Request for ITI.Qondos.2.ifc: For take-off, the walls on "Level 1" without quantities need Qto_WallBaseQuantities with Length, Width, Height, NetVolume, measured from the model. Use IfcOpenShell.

First a look at what the model holds.

```python
import ifcopenshell
import ifcopenshell.util.element
import ifcopenshell.util.unit

model = ifcopenshell.open("ITI.Qondos.2.ifc")
print(model.schema)
for unit_type in ("LENGTHUNIT", "AREAUNIT", "VOLUMEUNIT"):
    print(unit_type, ifcopenshell.util.unit.calculate_unit_scale(model, unit_type))
storey = next(s for s in model.by_type("IfcBuildingStorey") if s.Name == "Level 1")
walls = [e for e in ifcopenshell.util.element.get_decomposition(storey) if e.is_a("IfcWall")]
for e in sorted(walls, key=lambda e: e.id()):
    print(e.id(), e.is_a(), e.Name, list(ifcopenshell.util.element.get_psets(e, qtos_only=True)), sep=" | ")
```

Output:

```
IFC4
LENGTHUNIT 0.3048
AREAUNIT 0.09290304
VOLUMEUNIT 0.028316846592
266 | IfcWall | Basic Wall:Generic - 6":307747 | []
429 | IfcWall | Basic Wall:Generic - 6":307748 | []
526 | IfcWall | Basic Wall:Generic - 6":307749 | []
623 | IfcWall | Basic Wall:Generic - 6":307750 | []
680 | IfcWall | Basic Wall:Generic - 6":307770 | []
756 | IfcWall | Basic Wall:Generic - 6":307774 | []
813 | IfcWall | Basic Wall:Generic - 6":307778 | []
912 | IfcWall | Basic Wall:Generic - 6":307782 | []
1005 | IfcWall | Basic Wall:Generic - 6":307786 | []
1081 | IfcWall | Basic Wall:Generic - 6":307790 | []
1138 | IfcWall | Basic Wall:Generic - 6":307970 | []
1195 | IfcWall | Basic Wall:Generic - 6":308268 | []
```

```python
import ifcopenshell
import ifcopenshell.api.pset
import ifcopenshell.geom
import ifcopenshell.util.element
import ifcopenshell.util.shape
import ifcopenshell.util.unit

model = ifcopenshell.open("ITI.Qondos.2.ifc")
unit_scale = ifcopenshell.util.unit.calculate_unit_scale(model)
volume_scale = ifcopenshell.util.unit.calculate_unit_scale(model, "VOLUMEUNIT")
settings = ifcopenshell.geom.settings()

storey = next(s for s in model.by_type("IfcBuildingStorey") if s.Name == "Level 1")
walls = [e for e in ifcopenshell.util.element.get_decomposition(storey) if e.is_a("IfcWall")]

for e in sorted(walls, key=lambda e: e.id()):
    if ifcopenshell.util.element.get_psets(e, qtos_only=True, should_inherit=False):
        continue
    # Geometry comes back in metres, in the element's own axes.
    shape = ifcopenshell.geom.create_shape(settings, e)
    values = {
        "Length": ifcopenshell.util.shape.get_x(shape.geometry) / unit_scale,
        "Width": ifcopenshell.util.shape.get_y(shape.geometry) / unit_scale,
        "Height": ifcopenshell.util.shape.get_z(shape.geometry) / unit_scale,
        "NetVolume": ifcopenshell.util.shape.get_volume(shape.geometry) / volume_scale,
    }
    qto = ifcopenshell.api.pset.add_qto(model, product=e, name="Qto_WallBaseQuantities")
    ifcopenshell.api.pset.edit_qto(model, qto=qto, properties=values)
    print(e.id(), {k: round(v, 3) for k, v in values.items()})

model.write("ITI.Qondos.2_v2.ifc")
```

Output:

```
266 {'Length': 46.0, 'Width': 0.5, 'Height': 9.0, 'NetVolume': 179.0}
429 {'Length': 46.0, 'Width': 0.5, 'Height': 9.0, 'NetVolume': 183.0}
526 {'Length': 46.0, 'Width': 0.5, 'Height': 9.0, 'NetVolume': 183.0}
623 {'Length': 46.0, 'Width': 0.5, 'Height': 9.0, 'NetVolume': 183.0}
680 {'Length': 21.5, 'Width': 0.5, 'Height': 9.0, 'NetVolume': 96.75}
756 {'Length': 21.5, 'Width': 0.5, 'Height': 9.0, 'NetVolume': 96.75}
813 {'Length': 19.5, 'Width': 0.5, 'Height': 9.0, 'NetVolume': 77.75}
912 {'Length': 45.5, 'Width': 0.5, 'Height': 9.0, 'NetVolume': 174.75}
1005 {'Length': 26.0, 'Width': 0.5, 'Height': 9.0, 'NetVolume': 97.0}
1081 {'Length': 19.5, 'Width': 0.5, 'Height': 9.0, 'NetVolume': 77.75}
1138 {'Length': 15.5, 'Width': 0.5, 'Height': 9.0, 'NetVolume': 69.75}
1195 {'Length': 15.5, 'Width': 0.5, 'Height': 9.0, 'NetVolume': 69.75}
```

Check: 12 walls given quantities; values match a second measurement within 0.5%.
